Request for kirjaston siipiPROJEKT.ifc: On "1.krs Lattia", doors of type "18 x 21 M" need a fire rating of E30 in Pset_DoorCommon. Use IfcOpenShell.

First a look at what the model holds.

```python
import ifcopenshell
import ifcopenshell.util.element

model = ifcopenshell.open("kirjaston siipiPROJEKT.ifc")
print(model.schema)
storey = next(s for s in model.by_type("IfcBuildingStorey") if s.Name == "1.krs Lattia")
doors = [e for e in ifcopenshell.util.element.get_decomposition(storey) if e.is_a("IfcDoor")]
seen = {}
for e in doors:
    element_type = ifcopenshell.util.element.get_type(e)
    key = (element_type.Name if element_type != e and element_type else None, ifcopenshell.util.element.get_pset(e, "Pset_DoorCommon", "FireRating"))
    seen[key] = seen.get(key, 0) + 1
for (name, value), count in sorted(seen.items(), key=str):
    print(count, "x", name, "|", value)
```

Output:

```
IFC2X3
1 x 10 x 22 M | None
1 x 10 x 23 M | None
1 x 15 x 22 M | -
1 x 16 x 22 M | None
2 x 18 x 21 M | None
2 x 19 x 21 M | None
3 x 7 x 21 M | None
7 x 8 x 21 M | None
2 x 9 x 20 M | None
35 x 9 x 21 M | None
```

```python
import ifcopenshell
import ifcopenshell.api.pset
import ifcopenshell.util.element

model = ifcopenshell.open("kirjaston siipiPROJEKT.ifc")

storey = next(s for s in model.by_type("IfcBuildingStorey") if s.Name == "1.krs Lattia")
doors = [e for e in ifcopenshell.util.element.get_decomposition(storey) if e.is_a("IfcDoor")]

count = 0
for e in doors:
    element_type = ifcopenshell.util.element.get_type(e)
    if element_type in (None, e) or element_type.Name != "18 x 21 M":
        continue
    # add_pset returns the element's existing set when there is one.
    pset = ifcopenshell.api.pset.add_pset(model, product=e, name="Pset_DoorCommon")
    ifcopenshell.api.pset.edit_pset(model, pset=pset, properties={"FireRating": "E30"})
    count += 1

print(count, "doors updated")

model.write("kirjaston siipiPROJEKT-out.ifc")
```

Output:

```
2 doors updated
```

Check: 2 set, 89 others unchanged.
